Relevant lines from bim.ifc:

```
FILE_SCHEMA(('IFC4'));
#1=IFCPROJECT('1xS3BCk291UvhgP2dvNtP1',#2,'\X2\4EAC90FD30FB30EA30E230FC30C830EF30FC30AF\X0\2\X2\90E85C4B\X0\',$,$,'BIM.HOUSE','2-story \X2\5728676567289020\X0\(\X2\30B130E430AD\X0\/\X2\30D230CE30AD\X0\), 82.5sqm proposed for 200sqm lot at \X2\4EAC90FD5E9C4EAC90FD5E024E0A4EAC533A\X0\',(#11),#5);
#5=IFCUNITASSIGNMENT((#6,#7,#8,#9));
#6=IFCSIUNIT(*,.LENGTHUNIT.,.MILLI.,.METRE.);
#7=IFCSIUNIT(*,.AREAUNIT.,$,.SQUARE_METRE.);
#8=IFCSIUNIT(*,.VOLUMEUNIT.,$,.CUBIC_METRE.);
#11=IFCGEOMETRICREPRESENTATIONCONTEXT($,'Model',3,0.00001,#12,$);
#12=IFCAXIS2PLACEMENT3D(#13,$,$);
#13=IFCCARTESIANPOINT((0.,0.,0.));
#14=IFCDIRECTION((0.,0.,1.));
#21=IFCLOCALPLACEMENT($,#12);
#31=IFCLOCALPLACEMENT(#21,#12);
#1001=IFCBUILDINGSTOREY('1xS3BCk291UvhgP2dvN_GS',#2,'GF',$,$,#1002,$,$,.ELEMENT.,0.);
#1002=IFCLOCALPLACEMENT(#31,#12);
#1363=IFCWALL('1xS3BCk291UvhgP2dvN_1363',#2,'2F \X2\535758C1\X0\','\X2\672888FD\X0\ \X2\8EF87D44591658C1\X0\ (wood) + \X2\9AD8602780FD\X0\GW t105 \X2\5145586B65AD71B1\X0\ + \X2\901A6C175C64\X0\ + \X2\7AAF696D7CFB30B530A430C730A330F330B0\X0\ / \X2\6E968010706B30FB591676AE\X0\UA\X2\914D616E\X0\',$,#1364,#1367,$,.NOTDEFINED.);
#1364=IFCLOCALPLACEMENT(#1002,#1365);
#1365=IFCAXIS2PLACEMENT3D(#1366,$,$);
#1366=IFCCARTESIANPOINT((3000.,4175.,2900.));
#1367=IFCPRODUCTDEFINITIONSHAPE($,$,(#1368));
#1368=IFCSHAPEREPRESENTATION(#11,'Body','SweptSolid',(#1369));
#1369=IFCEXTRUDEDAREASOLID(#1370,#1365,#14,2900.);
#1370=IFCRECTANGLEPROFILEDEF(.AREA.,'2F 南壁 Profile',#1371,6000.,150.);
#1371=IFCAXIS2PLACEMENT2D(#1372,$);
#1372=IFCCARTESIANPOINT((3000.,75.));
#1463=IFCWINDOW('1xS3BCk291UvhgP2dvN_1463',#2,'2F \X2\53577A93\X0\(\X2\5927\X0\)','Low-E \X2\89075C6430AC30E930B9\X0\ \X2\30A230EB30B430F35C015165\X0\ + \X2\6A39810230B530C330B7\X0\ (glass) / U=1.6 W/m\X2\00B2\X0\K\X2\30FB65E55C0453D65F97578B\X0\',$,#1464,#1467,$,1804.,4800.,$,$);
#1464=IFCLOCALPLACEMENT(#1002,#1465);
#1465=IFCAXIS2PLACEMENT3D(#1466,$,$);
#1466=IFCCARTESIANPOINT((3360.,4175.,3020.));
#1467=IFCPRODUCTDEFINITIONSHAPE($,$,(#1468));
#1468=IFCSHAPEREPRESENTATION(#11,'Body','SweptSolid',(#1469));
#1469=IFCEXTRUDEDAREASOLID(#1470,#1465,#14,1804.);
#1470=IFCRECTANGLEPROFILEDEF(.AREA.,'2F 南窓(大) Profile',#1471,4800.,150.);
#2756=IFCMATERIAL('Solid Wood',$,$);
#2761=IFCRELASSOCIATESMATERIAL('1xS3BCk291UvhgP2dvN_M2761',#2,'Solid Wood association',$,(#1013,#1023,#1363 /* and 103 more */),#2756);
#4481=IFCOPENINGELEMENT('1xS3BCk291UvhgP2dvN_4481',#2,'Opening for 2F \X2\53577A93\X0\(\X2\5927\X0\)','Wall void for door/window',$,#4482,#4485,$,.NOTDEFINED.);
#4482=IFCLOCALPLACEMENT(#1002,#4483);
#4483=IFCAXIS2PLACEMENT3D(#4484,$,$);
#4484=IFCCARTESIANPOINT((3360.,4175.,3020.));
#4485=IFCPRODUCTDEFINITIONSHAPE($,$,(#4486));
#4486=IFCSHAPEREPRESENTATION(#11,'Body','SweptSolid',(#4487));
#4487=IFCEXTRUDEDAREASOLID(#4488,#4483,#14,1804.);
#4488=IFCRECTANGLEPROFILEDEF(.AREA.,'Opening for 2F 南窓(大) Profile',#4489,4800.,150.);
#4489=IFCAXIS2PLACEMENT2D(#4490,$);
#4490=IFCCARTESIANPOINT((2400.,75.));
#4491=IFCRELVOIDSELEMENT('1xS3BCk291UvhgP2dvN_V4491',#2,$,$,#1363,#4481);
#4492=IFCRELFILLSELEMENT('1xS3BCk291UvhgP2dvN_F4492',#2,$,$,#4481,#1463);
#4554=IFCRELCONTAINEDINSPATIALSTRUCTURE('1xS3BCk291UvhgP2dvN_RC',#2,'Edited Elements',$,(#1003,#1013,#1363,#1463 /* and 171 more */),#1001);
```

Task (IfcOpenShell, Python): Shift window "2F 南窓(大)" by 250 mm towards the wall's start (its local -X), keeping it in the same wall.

```python
import ifcopenshell
import ifcopenshell.api.geometry
import ifcopenshell.util.placement
import ifcopenshell.util.unit

model = ifcopenshell.open("bim.ifc")
unit_scale = ifcopenshell.util.unit.calculate_unit_scale(model)

window = model.by_id(1463)
opening = window.FillsVoids[0].RelatingOpeningElement
wall = opening.VoidsElements[0].RelatingBuildingElement

wall_matrix = ifcopenshell.util.placement.get_local_placement(wall.ObjectPlacement)
shift = wall_matrix[:3, 0] * -0.25 / unit_scale
before = ifcopenshell.util.placement.get_local_placement(window.ObjectPlacement)[:3, 3].copy()

# The window is not placed relative to its opening, so move both.
for product in (opening, window):
    matrix = ifcopenshell.util.placement.get_local_placement(product.ObjectPlacement)
    matrix[:3, 3] += shift
    ifcopenshell.api.geometry.edit_object_placement(model, product=product, matrix=matrix, is_si=False)

after = ifcopenshell.util.placement.get_local_placement(window.ObjectPlacement)[:3, 3]
print("window moved by", (after - before).round(3) + 0.0)

model.write("bim_edited.ifc")
```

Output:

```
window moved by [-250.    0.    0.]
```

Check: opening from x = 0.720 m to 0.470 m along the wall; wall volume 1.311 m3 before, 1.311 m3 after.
